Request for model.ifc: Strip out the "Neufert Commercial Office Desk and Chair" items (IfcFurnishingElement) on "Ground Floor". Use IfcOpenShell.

First a look at what the model holds.

```python
import ifcopenshell
import ifcopenshell.util.element

model = ifcopenshell.open("model.ifc")
print(model.schema)
storey = next(s for s in model.by_type("IfcBuildingStorey") if s.Name == "Ground Floor")
furniture = [e for e in ifcopenshell.util.element.get_decomposition(storey) if e.is_a("IfcFurnishingElement")]
seen = {}
for e in furniture:
    element_type = ifcopenshell.util.element.get_type(e)
    name = element_type.Name if element_type not in (None, e) else None
    seen[name] = seen.get(name, 0) + 1
for name, count in sorted(seen.items(), key=str):
    print(count, "x", name)
```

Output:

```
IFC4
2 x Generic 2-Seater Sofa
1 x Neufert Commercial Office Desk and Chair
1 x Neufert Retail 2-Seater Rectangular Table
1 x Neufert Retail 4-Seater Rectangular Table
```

```python
import ifcopenshell
import ifcopenshell.api.root
import ifcopenshell.util.element

model = ifcopenshell.open("model.ifc")

storey = next(s for s in model.by_type("IfcBuildingStorey") if s.Name == "Ground Floor")
furniture = [e for e in ifcopenshell.util.element.get_decomposition(storey) if e.is_a("IfcFurnishingElement")]
targets = [e for e in furniture if (t := ifcopenshell.util.element.get_type(e)) not in (None, e) and t.Name == "Neufert Commercial Office Desk and Chair"]

for e in targets:
    ifcopenshell.api.root.remove_product(model, product=e)
print(len(targets), "removed")

model.write("model_updated.ifc")
```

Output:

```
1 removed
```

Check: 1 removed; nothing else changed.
